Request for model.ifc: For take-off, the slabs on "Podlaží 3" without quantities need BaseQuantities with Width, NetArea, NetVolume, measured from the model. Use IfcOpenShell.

First a look at what the model holds.

```python
import ifcopenshell
import ifcopenshell.util.element
import ifcopenshell.util.unit

model = ifcopenshell.open("model.ifc")
print(model.schema)
for unit_type in ("LENGTHUNIT", "AREAUNIT", "VOLUMEUNIT"):
    print(unit_type, ifcopenshell.util.unit.calculate_unit_scale(model, unit_type))
storey = next(s for s in model.by_type("IfcBuildingStorey") if s.Name == "Podlaží 3")
slabs = [e for e in ifcopenshell.util.element.get_decomposition(storey) if e.is_a("IfcSlab")]
for e in sorted(slabs, key=lambda e: e.id()):
    print(e.id(), e.is_a(), e.Name, list(ifcopenshell.util.element.get_psets(e, qtos_only=True)), sep=" | ")
```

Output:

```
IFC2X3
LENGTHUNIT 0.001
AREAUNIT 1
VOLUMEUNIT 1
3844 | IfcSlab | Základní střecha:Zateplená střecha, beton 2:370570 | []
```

```python
import ifcopenshell
import ifcopenshell.api.pset
import ifcopenshell.geom
import ifcopenshell.util.element
import ifcopenshell.util.shape
import ifcopenshell.util.unit

model = ifcopenshell.open("model.ifc")
unit_scale = ifcopenshell.util.unit.calculate_unit_scale(model)
area_scale = ifcopenshell.util.unit.calculate_unit_scale(model, "AREAUNIT")
volume_scale = ifcopenshell.util.unit.calculate_unit_scale(model, "VOLUMEUNIT")
settings = ifcopenshell.geom.settings()

storey = next(s for s in model.by_type("IfcBuildingStorey") if s.Name == "Podlaží 3")
slabs = [e for e in ifcopenshell.util.element.get_decomposition(storey) if e.is_a("IfcSlab")]

for e in sorted(slabs, key=lambda e: e.id()):
    if ifcopenshell.util.element.get_psets(e, qtos_only=True, should_inherit=False):
        continue
    # Geometry comes back in metres, in the element's own axes.
    shape = ifcopenshell.geom.create_shape(settings, e)
    values = {
        "Width": ifcopenshell.util.shape.get_z(shape.geometry) / unit_scale,
        "NetArea": ifcopenshell.util.shape.get_footprint_area(shape.geometry) / area_scale,
        "NetVolume": ifcopenshell.util.shape.get_volume(shape.geometry) / volume_scale,
    }
    qto = ifcopenshell.api.pset.add_qto(model, product=e, name="BaseQuantities")
    ifcopenshell.api.pset.edit_qto(model, qto=qto, properties=values)
    print(e.id(), {k: round(v, 3) for k, v in values.items()})

model.write("model_edited.ifc")
```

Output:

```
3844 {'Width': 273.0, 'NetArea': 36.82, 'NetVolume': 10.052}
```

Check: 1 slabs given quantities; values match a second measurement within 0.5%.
